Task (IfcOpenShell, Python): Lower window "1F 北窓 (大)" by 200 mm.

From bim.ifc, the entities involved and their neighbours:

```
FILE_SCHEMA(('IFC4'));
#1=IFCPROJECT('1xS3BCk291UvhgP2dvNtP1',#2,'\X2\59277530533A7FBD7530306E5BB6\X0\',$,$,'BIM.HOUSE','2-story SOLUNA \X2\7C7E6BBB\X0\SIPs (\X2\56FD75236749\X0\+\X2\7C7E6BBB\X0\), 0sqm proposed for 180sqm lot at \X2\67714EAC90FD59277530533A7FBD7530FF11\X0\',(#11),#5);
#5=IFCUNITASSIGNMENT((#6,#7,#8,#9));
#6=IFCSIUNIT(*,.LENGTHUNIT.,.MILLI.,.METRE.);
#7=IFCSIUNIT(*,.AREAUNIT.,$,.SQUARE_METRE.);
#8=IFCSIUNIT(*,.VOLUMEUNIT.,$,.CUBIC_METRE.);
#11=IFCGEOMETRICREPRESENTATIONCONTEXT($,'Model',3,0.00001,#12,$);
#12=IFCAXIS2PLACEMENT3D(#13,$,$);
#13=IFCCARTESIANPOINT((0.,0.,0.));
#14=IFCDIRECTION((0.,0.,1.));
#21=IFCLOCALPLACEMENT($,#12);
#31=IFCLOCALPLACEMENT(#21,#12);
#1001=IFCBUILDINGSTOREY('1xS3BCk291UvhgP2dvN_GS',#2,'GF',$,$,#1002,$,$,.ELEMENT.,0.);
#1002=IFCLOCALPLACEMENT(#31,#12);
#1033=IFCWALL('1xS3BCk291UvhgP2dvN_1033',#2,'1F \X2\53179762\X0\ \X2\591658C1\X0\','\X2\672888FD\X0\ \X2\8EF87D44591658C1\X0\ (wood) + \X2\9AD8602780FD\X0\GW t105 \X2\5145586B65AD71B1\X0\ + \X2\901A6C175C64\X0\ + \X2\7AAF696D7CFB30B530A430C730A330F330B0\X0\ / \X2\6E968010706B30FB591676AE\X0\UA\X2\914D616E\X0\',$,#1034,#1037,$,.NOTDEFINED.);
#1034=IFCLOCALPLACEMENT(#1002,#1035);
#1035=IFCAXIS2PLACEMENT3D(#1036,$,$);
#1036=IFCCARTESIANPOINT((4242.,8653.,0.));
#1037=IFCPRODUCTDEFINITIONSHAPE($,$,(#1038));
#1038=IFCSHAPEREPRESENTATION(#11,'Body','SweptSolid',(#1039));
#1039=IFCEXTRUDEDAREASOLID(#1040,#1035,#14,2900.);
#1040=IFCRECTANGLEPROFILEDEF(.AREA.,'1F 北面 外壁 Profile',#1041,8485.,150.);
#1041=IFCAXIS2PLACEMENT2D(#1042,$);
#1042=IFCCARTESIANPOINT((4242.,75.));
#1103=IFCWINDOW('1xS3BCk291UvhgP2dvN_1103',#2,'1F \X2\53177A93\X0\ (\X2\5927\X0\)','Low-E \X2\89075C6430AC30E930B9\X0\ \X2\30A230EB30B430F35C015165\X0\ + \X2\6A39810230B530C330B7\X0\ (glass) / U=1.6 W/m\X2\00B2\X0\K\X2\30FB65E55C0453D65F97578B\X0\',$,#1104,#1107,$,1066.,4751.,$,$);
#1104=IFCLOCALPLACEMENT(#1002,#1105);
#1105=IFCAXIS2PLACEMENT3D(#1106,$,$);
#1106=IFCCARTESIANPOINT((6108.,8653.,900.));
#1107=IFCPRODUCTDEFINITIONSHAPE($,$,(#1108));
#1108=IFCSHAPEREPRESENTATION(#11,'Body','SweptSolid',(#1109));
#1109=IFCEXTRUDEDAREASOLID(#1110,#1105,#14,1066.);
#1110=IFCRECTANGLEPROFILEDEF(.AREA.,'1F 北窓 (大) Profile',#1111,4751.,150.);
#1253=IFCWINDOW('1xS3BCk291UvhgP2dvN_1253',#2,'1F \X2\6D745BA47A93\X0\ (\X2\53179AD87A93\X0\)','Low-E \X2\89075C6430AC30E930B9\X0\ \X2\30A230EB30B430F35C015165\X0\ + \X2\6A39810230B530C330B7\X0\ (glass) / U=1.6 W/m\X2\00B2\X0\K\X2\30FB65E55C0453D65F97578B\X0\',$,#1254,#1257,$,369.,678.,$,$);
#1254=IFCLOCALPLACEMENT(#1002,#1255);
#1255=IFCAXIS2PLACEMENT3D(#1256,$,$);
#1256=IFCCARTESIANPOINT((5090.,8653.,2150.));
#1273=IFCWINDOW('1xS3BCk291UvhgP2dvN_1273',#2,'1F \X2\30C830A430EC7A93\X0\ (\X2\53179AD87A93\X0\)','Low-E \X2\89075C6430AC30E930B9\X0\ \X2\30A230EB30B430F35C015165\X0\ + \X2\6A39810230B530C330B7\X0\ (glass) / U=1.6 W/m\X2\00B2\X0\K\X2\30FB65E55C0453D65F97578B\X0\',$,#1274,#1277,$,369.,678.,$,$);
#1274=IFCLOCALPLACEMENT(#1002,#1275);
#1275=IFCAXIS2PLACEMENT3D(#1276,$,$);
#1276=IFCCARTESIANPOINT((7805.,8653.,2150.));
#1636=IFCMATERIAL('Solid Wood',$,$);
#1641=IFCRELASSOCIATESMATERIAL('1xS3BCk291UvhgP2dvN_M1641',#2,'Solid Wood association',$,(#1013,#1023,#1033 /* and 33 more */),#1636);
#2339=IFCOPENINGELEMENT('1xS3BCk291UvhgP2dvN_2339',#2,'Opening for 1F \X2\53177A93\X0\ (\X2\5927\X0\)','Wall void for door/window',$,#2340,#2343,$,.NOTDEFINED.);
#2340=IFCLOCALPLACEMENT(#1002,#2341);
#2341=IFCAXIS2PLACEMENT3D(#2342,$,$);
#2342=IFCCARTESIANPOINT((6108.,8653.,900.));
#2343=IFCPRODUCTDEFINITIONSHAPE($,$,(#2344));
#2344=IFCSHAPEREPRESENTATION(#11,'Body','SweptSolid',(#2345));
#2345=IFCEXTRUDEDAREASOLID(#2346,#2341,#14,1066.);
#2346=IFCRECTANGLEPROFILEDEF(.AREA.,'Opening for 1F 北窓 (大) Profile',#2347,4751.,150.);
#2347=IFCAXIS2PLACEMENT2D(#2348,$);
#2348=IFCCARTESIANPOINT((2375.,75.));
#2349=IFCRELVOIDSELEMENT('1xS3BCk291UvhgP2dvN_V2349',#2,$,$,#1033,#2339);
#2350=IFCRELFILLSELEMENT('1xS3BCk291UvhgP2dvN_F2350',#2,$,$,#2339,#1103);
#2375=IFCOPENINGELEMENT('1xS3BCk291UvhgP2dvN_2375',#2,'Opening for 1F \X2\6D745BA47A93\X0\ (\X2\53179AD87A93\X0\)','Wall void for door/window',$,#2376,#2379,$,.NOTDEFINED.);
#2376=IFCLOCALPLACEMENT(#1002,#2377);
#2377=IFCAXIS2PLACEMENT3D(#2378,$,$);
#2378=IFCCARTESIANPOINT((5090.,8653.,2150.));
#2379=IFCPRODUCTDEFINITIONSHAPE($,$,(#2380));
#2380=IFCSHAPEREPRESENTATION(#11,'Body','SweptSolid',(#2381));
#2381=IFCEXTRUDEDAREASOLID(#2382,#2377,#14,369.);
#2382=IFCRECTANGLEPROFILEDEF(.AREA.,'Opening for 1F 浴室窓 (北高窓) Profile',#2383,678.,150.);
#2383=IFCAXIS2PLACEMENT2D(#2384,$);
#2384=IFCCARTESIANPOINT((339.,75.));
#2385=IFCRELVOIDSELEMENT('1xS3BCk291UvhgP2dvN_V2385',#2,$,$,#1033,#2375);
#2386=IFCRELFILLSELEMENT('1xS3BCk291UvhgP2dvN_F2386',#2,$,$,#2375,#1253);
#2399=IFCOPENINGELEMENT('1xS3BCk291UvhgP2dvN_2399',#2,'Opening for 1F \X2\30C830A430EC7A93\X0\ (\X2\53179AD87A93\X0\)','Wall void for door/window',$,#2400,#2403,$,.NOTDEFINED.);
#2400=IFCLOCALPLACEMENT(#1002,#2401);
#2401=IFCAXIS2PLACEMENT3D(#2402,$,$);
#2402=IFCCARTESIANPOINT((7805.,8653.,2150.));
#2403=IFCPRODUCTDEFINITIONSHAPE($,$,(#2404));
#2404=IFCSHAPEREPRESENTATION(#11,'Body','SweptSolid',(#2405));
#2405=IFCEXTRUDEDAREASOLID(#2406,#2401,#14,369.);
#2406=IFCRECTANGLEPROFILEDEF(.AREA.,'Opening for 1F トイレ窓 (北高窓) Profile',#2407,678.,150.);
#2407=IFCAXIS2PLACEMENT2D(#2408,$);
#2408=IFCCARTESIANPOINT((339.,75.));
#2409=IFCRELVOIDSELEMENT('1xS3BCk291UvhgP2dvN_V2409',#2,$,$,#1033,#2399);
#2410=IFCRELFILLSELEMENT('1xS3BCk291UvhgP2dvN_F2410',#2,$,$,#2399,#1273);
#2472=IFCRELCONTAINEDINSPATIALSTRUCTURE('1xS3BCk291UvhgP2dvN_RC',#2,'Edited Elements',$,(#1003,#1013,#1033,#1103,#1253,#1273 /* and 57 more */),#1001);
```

```python
import numpy as np
import ifcopenshell
import ifcopenshell.api.geometry
import ifcopenshell.util.placement
import ifcopenshell.util.unit

model = ifcopenshell.open("bim.ifc")
unit_scale = ifcopenshell.util.unit.calculate_unit_scale(model)

window = model.by_guid("1xS3BCk291UvhgP2dvN_1103")
opening = window.FillsVoids[0].RelatingOpeningElement
dz = -0.2 / unit_scale

shift = np.array([0.0, 0.0, dz])
# The window is not placed relative to its opening, so move both.
for product in (opening, window):
    matrix = ifcopenshell.util.placement.get_local_placement(product.ObjectPlacement)
    matrix[:3, 3] += shift
    ifcopenshell.api.geometry.edit_object_placement(model, product=product, matrix=matrix, is_si=False)

print(f"moved by {dz * unit_scale:+.3f} m")

model.write("bim_edited.ifc")
```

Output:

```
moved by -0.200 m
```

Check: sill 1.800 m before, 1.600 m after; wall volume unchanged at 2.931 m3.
